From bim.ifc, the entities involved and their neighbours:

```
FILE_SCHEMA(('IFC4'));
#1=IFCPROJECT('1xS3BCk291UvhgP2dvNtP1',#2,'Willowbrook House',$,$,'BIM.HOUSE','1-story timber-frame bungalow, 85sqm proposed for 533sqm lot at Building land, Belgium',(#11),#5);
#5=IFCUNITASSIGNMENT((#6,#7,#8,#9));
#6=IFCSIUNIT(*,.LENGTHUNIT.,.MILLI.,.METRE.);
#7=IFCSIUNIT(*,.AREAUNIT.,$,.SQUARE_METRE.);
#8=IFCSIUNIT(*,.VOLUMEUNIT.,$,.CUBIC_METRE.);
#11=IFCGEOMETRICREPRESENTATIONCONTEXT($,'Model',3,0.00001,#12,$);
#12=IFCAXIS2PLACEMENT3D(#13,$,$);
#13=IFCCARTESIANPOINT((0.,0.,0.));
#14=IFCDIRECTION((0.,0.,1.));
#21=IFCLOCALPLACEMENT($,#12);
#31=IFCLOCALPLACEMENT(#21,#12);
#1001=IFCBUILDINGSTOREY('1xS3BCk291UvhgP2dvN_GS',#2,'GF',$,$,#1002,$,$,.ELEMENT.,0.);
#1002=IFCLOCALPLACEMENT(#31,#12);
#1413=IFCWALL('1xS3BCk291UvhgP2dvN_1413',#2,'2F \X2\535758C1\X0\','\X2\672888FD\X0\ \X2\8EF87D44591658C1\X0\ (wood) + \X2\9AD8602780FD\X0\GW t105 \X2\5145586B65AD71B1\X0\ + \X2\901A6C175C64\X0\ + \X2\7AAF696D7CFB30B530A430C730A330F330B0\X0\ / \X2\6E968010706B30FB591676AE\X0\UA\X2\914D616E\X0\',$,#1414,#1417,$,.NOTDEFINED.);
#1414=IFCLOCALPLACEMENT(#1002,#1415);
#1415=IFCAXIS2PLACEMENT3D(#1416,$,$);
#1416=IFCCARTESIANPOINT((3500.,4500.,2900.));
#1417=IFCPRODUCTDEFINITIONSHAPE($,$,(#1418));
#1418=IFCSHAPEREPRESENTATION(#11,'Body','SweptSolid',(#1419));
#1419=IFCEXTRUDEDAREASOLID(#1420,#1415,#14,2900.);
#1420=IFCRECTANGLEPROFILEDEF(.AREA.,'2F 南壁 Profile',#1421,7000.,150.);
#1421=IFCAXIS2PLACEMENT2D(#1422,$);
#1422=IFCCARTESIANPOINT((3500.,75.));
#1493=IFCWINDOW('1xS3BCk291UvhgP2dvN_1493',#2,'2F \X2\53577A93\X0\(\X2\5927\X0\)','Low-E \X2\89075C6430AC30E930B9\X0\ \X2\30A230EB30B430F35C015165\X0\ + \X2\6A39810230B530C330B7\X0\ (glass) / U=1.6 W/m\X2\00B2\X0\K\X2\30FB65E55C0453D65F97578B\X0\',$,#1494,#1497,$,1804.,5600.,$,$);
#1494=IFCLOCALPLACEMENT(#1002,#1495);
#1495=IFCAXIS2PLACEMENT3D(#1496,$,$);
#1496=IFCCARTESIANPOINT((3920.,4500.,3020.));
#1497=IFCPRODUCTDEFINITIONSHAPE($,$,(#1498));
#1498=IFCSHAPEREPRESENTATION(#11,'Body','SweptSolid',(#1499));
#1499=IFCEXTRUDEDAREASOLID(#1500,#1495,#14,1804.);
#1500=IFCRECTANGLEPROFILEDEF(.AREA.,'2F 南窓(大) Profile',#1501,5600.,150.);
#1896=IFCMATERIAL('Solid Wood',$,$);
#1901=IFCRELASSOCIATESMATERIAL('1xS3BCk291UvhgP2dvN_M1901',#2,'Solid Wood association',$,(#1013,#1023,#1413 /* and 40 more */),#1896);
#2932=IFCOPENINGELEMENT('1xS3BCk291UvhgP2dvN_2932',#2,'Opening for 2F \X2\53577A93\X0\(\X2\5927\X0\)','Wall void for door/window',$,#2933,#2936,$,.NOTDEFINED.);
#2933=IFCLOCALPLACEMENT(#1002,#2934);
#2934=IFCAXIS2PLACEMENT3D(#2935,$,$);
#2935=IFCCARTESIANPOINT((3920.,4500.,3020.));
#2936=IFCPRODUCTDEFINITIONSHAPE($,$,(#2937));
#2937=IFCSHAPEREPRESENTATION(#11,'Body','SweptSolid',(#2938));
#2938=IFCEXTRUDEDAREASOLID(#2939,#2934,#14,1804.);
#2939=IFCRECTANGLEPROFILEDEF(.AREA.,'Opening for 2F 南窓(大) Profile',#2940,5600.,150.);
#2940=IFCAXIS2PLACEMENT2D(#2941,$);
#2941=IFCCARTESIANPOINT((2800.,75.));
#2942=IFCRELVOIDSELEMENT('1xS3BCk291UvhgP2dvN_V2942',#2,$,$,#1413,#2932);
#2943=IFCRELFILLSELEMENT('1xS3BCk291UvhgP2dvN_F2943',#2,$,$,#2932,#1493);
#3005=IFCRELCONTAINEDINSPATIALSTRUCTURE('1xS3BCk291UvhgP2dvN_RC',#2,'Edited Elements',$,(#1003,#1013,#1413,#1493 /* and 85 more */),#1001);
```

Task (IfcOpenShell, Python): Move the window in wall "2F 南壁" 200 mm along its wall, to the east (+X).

```python
import ifcopenshell
import ifcopenshell.api.geometry
import ifcopenshell.util.placement
import ifcopenshell.util.unit

model = ifcopenshell.open("bim.ifc")
unit_scale = ifcopenshell.util.unit.calculate_unit_scale(model)

window = model.by_guid("1xS3BCk291UvhgP2dvN_1493")
opening = window.FillsVoids[0].RelatingOpeningElement
wall = opening.VoidsElements[0].RelatingBuildingElement

wall_matrix = ifcopenshell.util.placement.get_local_placement(wall.ObjectPlacement)
shift = wall_matrix[:3, 0] * 0.2 / unit_scale
before = ifcopenshell.util.placement.get_local_placement(window.ObjectPlacement)[:3, 3].copy()

# The window is not placed relative to its opening, so move both.
for product in (opening, window):
    matrix = ifcopenshell.util.placement.get_local_placement(product.ObjectPlacement)
    matrix[:3, 3] += shift
    ifcopenshell.api.geometry.edit_object_placement(model, product=product, matrix=matrix, is_si=False)

after = ifcopenshell.util.placement.get_local_placement(window.ObjectPlacement)[:3, 3]
print("window moved by", (after - before).round(3) + 0.0)

model.write("bim-out.ifc")
```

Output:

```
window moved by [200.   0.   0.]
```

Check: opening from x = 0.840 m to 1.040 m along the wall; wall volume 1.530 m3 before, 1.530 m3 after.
